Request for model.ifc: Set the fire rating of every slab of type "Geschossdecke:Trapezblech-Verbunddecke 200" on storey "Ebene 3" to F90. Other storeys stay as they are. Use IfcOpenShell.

First a look at what the model holds.

```python
import ifcopenshell
import ifcopenshell.util.element

model = ifcopenshell.open("model.ifc")
print(model.schema)
storey = next(s for s in model.by_type("IfcBuildingStorey") if s.Name == "Ebene 3")
slabs = [e for e in ifcopenshell.util.element.get_decomposition(storey) if e.is_a("IfcSlab")]
seen = {}
for e in slabs:
    element_type = ifcopenshell.util.element.get_type(e)
    key = (element_type.Name if element_type != e and element_type else None, ifcopenshell.util.element.get_pset(e, "Pset_SlabCommon", "FireRating"))
    seen[key] = seen.get(key, 0) + 1
for (name, value), count in sorted(seen.items(), key=str):
    print(count, "x", name, "|", value)
```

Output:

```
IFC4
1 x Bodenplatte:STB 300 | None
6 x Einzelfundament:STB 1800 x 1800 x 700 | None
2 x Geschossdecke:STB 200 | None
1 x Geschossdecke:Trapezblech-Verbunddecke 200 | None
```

```python
import ifcopenshell
import ifcopenshell.api.pset
import ifcopenshell.util.element

model = ifcopenshell.open("model.ifc")

storey = next(s for s in model.by_type("IfcBuildingStorey") if s.Name == "Ebene 3")
slabs = [e for e in ifcopenshell.util.element.get_decomposition(storey) if e.is_a("IfcSlab")]

count = 0
for e in slabs:
    element_type = ifcopenshell.util.element.get_type(e)
    if element_type in (None, e) or element_type.Name != "Geschossdecke:Trapezblech-Verbunddecke 200":
        continue
    # add_pset returns the element's existing set when there is one.
    pset = ifcopenshell.api.pset.add_pset(model, product=e, name="Pset_SlabCommon")
    ifcopenshell.api.pset.edit_pset(model, pset=pset, properties={"FireRating": "F90"})
    count += 1

print(count, "slabs updated")

model.write("model_v2.ifc")
```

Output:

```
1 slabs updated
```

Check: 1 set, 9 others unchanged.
